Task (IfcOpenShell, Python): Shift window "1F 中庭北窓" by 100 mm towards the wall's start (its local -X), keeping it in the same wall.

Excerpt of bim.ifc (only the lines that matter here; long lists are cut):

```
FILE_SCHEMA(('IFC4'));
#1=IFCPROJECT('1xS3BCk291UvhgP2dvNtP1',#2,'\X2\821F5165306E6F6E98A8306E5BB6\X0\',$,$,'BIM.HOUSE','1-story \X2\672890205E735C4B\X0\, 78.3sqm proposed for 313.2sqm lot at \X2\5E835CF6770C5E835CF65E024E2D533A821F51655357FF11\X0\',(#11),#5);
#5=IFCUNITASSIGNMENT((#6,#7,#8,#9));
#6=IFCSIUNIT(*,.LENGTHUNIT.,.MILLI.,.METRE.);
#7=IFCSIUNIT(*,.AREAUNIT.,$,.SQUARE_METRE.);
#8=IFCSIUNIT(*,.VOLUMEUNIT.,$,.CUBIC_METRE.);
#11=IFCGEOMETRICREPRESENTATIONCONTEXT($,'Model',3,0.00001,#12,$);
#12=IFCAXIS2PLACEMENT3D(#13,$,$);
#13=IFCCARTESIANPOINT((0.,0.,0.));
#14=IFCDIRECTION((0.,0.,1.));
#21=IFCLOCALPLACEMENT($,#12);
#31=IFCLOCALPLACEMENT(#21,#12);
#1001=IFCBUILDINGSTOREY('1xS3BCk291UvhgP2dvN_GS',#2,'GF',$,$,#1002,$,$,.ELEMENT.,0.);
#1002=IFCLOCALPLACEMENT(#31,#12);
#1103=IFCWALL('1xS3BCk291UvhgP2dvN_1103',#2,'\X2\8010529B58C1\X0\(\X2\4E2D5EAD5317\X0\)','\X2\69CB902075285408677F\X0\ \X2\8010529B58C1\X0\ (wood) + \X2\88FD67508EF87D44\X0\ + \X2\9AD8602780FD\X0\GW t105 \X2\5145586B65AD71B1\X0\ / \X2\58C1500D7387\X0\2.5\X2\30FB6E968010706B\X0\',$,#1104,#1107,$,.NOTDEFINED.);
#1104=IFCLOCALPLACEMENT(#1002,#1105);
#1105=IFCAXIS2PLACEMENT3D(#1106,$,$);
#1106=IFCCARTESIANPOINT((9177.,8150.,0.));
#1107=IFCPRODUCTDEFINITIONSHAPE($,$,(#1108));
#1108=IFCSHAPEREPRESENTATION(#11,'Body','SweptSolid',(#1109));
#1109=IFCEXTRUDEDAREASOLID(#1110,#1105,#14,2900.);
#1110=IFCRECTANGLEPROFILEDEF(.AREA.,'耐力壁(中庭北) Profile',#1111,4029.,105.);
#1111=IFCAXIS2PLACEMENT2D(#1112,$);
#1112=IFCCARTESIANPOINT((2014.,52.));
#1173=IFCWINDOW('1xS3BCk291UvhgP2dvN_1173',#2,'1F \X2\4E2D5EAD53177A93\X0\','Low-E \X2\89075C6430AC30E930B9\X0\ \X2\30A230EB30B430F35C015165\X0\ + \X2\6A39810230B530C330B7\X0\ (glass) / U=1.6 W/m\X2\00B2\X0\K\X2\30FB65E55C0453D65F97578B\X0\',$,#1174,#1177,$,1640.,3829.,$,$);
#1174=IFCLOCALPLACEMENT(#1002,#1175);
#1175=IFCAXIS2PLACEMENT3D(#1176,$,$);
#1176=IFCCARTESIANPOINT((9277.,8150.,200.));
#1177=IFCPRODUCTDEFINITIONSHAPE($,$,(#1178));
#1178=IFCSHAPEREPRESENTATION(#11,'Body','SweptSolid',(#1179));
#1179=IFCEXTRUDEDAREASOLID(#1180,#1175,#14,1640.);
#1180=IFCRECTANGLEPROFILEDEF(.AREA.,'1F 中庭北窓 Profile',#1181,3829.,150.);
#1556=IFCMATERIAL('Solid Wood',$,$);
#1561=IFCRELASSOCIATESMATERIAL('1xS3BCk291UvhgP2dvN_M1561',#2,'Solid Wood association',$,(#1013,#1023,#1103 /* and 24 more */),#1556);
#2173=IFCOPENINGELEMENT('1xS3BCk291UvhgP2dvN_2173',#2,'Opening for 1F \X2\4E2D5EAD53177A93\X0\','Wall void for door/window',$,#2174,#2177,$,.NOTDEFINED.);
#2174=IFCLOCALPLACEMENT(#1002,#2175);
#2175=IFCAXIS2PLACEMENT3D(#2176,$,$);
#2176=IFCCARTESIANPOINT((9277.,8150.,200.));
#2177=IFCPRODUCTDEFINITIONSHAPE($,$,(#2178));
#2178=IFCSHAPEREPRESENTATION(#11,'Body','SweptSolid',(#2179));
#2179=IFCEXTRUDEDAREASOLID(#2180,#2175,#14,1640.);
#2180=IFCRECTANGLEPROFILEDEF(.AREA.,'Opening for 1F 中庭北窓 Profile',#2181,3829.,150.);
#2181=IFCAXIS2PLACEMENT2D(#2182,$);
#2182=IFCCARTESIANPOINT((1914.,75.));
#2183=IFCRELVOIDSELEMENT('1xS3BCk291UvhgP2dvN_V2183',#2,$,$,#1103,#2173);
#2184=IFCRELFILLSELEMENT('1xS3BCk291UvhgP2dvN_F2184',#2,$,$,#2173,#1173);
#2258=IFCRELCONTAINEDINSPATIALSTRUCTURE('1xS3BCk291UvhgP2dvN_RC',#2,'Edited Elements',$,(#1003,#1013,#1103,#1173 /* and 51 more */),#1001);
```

```python
import ifcopenshell
import ifcopenshell.api.geometry
import ifcopenshell.util.placement
import ifcopenshell.util.unit

model = ifcopenshell.open("bim.ifc")
unit_scale = ifcopenshell.util.unit.calculate_unit_scale(model)

window = model.by_id(1173)
opening = window.FillsVoids[0].RelatingOpeningElement
wall = opening.VoidsElements[0].RelatingBuildingElement

wall_matrix = ifcopenshell.util.placement.get_local_placement(wall.ObjectPlacement)
shift = wall_matrix[:3, 0] * -0.1 / unit_scale
before = ifcopenshell.util.placement.get_local_placement(window.ObjectPlacement)[:3, 3].copy()

# The window is not placed relative to its opening, so move both.
for product in (opening, window):
    matrix = ifcopenshell.util.placement.get_local_placement(product.ObjectPlacement)
    matrix[:3, 3] += shift
    ifcopenshell.api.geometry.edit_object_placement(model, product=product, matrix=matrix, is_si=False)

after = ifcopenshell.util.placement.get_local_placement(window.ObjectPlacement)[:3, 3]
print("window moved by", (after - before).round(3) + 0.0)

model.write("bim_rev.ifc")
```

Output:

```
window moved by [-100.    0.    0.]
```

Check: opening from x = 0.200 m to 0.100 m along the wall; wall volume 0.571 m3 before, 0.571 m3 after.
